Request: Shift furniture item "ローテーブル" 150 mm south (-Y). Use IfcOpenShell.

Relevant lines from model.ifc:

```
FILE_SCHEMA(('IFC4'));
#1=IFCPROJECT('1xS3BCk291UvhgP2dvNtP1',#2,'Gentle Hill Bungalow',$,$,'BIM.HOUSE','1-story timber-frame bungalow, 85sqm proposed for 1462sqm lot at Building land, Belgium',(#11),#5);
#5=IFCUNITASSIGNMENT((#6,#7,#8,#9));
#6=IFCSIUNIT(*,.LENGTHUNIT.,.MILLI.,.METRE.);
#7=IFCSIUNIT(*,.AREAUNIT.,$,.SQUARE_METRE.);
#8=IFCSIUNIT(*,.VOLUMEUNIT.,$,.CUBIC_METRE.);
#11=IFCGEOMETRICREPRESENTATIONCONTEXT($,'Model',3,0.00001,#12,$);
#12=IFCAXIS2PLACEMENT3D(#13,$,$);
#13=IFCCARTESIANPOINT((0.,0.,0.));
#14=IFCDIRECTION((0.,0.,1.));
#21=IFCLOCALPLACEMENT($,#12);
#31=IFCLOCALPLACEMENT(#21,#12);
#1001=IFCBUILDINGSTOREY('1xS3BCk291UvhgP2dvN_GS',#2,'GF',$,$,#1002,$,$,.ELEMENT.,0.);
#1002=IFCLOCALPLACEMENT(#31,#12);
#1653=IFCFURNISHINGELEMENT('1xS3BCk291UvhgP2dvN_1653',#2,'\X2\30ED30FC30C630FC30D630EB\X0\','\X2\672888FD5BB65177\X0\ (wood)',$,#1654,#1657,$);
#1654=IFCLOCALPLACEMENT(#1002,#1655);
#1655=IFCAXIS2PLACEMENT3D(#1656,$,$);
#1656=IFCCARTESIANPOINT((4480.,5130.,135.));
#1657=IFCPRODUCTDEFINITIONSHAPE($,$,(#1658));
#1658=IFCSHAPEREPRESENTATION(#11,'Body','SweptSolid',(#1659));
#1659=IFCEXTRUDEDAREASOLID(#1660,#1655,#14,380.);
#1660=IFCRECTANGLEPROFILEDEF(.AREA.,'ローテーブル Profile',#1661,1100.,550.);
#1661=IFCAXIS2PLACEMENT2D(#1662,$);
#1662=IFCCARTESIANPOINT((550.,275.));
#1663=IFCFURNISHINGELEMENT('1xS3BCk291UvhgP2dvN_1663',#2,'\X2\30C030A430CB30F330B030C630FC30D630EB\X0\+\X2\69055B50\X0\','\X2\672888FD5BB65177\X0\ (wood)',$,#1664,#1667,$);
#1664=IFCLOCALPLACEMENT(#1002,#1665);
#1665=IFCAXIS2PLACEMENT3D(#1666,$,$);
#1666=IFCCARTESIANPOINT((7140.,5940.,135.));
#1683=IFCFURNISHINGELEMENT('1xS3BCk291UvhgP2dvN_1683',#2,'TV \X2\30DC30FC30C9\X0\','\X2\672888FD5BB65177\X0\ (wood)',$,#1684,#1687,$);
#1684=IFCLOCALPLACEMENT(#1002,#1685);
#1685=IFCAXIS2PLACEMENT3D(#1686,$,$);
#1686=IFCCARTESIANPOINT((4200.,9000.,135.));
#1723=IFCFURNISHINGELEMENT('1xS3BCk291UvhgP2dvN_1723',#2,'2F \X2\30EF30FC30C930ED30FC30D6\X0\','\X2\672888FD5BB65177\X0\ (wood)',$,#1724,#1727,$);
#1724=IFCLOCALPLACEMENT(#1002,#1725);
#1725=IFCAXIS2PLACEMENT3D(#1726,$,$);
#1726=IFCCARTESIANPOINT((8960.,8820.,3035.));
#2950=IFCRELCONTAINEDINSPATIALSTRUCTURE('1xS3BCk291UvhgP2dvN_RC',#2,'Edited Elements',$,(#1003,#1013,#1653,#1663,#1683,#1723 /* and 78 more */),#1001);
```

```python
import ifcopenshell
import ifcopenshell.api.geometry
import ifcopenshell.util.placement
import ifcopenshell.util.unit

model = ifcopenshell.open("model.ifc")
unit_scale = ifcopenshell.util.unit.calculate_unit_scale(model)

item = model.by_guid("1xS3BCk291UvhgP2dvN_1653")
matrix = ifcopenshell.util.placement.get_local_placement(item.ObjectPlacement)
matrix[1, 3] -= 0.15 / unit_scale
ifcopenshell.api.geometry.edit_object_placement(model, product=item, matrix=matrix, is_si=False)

print(ifcopenshell.util.placement.get_local_placement(item.ObjectPlacement).round(3) + 0.0)

model.write("model-out.ifc")
```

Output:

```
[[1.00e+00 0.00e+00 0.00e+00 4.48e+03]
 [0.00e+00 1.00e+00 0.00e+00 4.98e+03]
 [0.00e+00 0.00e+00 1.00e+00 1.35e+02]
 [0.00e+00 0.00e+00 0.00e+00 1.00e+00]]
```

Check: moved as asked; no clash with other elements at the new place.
